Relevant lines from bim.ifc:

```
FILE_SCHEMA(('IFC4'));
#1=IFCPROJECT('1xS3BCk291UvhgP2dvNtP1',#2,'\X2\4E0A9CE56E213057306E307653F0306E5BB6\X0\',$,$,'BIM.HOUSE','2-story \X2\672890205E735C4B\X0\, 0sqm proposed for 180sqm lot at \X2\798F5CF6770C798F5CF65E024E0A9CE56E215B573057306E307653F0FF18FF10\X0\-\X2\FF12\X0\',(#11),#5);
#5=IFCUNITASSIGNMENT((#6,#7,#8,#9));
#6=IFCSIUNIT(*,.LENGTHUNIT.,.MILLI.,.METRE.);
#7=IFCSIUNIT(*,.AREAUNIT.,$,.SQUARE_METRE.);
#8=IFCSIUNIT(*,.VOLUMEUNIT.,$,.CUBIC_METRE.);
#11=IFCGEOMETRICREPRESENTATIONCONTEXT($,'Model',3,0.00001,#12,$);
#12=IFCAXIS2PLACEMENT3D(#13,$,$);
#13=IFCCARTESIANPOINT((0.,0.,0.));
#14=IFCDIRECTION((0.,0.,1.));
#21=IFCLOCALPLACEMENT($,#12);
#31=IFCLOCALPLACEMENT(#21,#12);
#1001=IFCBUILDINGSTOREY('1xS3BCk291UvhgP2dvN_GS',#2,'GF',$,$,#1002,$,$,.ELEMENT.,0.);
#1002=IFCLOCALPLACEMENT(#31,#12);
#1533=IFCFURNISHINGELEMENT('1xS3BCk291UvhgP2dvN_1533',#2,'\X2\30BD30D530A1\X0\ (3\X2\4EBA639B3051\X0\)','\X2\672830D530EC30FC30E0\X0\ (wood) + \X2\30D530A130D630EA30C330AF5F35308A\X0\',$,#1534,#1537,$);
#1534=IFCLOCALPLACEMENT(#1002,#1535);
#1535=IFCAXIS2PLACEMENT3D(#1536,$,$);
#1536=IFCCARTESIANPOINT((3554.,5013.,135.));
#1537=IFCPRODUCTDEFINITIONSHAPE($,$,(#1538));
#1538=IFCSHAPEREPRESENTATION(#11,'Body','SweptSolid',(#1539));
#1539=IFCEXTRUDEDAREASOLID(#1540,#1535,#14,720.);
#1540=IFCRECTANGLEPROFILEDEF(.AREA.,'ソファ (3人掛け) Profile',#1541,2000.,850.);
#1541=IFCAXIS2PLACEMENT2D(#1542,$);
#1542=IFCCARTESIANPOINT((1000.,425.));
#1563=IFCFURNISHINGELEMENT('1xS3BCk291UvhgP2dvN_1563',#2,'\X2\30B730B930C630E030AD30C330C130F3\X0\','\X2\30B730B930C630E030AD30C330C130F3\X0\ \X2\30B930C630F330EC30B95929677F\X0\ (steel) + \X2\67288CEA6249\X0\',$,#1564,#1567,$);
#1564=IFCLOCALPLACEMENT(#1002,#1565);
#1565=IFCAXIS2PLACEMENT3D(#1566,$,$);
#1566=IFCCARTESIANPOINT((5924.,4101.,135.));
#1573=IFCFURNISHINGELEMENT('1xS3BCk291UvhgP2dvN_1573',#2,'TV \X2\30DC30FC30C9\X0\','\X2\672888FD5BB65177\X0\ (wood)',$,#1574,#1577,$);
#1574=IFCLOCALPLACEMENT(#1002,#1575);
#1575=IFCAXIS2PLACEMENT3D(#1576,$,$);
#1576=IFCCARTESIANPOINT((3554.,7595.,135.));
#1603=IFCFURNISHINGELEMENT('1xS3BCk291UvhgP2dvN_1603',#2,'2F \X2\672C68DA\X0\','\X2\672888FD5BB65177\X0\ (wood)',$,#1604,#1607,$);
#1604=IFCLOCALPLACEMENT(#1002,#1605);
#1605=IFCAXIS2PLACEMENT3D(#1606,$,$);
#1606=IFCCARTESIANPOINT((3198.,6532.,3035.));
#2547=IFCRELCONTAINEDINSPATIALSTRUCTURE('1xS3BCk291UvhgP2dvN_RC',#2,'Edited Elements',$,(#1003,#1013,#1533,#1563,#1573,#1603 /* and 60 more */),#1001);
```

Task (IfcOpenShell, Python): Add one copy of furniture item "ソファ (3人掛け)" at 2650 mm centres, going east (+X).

```python
import numpy as np
import ifcopenshell
import ifcopenshell.api.geometry
import ifcopenshell.api.root
import ifcopenshell.util.element
import ifcopenshell.util.placement

model = ifcopenshell.open("bim.ifc")


def reuse_history(source, copy):
    """copy_class also copies each property set's owner history, people and application; keep the originals."""
    for rel in copy.IsDefinedBy:
        if rel.is_a("IfcRelDefinesByProperties") and (history := rel.RelatingPropertyDefinition.OwnerHistory):
            rel.RelatingPropertyDefinition.OwnerHistory = source.OwnerHistory
            ifcopenshell.util.element.remove_deep2(model, history)


source = model.by_guid("1xS3BCk291UvhgP2dvN_1533")
base = ifcopenshell.util.placement.get_local_placement(source.ObjectPlacement)
step = np.array([1.0, 0.0, 0.0]) * 2650.0

for i in range(1, 2):
    copy = ifcopenshell.api.root.copy_class(model, product=source)
    copy.Representation = ifcopenshell.util.element.copy_deep(
        model, source.Representation, exclude=["IfcGeometricRepresentationContext", "IfcRepresentationMap"]
    )
    reuse_history(source, copy)
    matrix = base.copy()
    matrix[:3, 3] += i * step
    print("added at", matrix[:3, 3].round(3) + 0.0)
    ifcopenshell.api.geometry.edit_object_placement(model, product=copy, matrix=matrix, is_si=False)

model.write("bim-out.ifc")
```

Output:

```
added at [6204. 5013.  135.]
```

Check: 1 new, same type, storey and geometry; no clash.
